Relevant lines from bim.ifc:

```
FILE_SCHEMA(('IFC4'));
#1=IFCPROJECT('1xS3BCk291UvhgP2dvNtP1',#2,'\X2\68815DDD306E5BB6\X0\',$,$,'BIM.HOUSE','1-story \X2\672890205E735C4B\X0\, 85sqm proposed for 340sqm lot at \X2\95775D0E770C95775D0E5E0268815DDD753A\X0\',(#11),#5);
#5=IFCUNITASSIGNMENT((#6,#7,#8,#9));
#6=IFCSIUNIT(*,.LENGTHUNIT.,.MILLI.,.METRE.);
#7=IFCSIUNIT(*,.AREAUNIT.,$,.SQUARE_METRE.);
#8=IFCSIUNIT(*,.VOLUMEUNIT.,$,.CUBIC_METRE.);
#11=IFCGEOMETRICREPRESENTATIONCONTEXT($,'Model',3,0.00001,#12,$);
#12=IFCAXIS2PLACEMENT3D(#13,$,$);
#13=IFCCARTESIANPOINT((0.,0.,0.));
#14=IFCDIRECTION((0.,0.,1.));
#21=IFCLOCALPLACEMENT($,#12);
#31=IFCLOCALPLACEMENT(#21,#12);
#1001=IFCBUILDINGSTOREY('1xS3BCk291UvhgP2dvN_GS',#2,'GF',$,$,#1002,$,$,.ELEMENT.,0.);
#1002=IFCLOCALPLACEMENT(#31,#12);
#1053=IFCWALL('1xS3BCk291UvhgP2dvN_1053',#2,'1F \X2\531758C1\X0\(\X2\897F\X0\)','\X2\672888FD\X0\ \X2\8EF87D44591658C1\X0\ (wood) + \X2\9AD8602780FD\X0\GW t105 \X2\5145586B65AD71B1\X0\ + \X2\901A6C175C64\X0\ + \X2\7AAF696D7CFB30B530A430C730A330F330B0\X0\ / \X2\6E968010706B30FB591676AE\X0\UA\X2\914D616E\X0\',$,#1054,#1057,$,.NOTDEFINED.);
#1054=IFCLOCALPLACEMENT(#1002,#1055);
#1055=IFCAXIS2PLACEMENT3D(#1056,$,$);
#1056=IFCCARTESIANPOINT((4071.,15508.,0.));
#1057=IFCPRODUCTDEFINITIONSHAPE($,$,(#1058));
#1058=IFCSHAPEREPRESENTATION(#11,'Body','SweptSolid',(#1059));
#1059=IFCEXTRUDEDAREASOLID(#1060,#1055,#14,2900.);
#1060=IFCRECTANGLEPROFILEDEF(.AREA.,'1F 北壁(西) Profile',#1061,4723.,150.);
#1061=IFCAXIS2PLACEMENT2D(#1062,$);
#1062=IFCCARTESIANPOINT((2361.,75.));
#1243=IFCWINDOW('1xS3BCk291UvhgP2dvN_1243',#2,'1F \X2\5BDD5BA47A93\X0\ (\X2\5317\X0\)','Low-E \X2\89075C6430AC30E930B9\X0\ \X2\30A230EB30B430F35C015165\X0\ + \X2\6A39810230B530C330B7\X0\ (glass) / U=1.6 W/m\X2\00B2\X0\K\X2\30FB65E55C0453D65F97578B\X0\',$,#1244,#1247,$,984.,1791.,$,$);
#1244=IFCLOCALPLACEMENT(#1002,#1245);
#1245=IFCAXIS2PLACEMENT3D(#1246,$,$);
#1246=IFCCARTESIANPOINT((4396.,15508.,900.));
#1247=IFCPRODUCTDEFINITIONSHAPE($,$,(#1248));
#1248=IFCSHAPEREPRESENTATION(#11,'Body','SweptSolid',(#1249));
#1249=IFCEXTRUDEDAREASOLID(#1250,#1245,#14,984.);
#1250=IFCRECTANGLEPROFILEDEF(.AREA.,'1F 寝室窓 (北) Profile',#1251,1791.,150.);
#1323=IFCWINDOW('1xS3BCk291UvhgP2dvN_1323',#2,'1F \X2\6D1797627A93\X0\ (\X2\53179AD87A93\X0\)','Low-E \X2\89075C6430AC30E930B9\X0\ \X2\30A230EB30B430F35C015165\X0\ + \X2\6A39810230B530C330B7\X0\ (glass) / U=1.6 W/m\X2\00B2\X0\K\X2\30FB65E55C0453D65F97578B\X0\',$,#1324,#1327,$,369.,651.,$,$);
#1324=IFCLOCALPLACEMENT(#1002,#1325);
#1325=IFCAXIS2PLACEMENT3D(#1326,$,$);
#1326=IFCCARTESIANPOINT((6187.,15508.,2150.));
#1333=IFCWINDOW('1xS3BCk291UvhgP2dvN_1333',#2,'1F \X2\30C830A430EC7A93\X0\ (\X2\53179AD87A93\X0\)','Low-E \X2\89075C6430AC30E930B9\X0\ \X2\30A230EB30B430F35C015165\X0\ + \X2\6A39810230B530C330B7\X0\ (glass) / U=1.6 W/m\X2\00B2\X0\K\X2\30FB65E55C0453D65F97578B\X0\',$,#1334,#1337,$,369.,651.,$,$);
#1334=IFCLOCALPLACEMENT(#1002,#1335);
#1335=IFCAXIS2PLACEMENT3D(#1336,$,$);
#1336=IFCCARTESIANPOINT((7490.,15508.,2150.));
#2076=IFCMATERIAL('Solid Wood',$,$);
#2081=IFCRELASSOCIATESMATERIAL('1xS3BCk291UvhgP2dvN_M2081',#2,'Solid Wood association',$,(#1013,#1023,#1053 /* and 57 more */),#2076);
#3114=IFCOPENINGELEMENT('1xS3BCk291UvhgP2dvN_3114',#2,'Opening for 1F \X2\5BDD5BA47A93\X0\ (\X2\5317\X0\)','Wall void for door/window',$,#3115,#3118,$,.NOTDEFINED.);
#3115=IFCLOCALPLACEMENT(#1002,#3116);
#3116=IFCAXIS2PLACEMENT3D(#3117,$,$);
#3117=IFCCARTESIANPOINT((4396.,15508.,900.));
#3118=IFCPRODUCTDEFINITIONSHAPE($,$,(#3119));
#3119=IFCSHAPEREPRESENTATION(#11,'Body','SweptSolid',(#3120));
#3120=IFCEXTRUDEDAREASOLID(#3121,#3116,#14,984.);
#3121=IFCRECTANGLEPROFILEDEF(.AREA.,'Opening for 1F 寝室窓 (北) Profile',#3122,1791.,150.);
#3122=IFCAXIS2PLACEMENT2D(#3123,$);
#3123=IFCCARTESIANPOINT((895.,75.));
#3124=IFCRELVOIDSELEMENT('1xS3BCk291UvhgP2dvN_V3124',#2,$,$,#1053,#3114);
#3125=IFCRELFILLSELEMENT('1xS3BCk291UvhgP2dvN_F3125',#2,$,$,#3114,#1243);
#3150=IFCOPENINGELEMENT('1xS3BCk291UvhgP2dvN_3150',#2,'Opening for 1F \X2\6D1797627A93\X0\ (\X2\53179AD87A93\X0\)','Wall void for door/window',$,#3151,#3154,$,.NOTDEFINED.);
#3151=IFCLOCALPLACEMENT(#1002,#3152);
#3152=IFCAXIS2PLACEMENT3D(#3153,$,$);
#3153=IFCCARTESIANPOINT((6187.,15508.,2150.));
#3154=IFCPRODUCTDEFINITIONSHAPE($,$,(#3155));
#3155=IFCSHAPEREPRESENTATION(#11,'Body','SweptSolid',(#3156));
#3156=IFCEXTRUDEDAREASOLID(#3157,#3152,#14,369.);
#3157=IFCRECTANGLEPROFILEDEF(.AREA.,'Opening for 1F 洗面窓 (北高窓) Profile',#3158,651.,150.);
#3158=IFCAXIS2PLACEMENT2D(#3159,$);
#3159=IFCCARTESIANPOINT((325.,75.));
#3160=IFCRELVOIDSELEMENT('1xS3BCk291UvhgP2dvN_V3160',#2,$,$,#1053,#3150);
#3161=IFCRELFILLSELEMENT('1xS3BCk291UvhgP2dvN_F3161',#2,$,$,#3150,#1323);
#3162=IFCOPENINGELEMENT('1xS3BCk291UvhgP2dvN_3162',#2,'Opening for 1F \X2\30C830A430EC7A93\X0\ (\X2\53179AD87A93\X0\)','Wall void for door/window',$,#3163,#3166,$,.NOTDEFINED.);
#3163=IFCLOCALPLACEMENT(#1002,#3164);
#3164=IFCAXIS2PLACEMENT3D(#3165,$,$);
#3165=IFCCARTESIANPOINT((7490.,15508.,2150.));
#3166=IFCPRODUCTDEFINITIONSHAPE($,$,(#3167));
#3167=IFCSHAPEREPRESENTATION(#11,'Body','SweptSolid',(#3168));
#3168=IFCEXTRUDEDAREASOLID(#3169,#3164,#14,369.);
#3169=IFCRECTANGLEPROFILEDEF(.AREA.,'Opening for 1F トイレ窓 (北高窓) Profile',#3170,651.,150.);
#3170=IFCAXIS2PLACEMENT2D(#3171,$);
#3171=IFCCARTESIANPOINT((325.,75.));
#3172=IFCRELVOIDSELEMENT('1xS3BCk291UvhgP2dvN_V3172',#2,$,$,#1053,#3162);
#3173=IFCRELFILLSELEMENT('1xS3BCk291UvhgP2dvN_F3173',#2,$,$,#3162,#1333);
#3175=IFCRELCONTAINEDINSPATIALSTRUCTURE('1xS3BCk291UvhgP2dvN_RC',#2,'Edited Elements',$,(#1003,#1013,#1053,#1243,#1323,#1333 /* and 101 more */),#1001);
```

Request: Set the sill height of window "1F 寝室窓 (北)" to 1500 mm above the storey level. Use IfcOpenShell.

```python
import numpy as np
import ifcopenshell
import ifcopenshell.api.geometry
import ifcopenshell.geom
import ifcopenshell.util.element
import ifcopenshell.util.placement
import ifcopenshell.util.shape
import ifcopenshell.util.unit

model = ifcopenshell.open("bim.ifc")
unit_scale = ifcopenshell.util.unit.calculate_unit_scale(model)

window = model.by_guid("1xS3BCk291UvhgP2dvN_1243")
opening = window.FillsVoids[0].RelatingOpeningElement
storey = ifcopenshell.util.element.get_container(window, ifc_class="IfcBuildingStorey")
level = ifcopenshell.util.placement.get_local_placement(storey.ObjectPlacement)[2, 3]

# The opening's origin need not be at the sill, so measure its lowest point.
shape = ifcopenshell.geom.create_shape(ifcopenshell.geom.settings(), opening)
bottom = ifcopenshell.util.shape.get_shape_bottom_elevation(shape, shape.geometry) / unit_scale
dz = level + 1500.0 - bottom

shift = np.array([0.0, 0.0, dz])
# The window is not placed relative to its opening, so move both.
for product in (opening, window):
    matrix = ifcopenshell.util.placement.get_local_placement(product.ObjectPlacement)
    matrix[:3, 3] += shift
    ifcopenshell.api.geometry.edit_object_placement(model, product=product, matrix=matrix, is_si=False)

print(f"moved by {dz * unit_scale:+.3f} m")

model.write("bim_edited.ifc")
```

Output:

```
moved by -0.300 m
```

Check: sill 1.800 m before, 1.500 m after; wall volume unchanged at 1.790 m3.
